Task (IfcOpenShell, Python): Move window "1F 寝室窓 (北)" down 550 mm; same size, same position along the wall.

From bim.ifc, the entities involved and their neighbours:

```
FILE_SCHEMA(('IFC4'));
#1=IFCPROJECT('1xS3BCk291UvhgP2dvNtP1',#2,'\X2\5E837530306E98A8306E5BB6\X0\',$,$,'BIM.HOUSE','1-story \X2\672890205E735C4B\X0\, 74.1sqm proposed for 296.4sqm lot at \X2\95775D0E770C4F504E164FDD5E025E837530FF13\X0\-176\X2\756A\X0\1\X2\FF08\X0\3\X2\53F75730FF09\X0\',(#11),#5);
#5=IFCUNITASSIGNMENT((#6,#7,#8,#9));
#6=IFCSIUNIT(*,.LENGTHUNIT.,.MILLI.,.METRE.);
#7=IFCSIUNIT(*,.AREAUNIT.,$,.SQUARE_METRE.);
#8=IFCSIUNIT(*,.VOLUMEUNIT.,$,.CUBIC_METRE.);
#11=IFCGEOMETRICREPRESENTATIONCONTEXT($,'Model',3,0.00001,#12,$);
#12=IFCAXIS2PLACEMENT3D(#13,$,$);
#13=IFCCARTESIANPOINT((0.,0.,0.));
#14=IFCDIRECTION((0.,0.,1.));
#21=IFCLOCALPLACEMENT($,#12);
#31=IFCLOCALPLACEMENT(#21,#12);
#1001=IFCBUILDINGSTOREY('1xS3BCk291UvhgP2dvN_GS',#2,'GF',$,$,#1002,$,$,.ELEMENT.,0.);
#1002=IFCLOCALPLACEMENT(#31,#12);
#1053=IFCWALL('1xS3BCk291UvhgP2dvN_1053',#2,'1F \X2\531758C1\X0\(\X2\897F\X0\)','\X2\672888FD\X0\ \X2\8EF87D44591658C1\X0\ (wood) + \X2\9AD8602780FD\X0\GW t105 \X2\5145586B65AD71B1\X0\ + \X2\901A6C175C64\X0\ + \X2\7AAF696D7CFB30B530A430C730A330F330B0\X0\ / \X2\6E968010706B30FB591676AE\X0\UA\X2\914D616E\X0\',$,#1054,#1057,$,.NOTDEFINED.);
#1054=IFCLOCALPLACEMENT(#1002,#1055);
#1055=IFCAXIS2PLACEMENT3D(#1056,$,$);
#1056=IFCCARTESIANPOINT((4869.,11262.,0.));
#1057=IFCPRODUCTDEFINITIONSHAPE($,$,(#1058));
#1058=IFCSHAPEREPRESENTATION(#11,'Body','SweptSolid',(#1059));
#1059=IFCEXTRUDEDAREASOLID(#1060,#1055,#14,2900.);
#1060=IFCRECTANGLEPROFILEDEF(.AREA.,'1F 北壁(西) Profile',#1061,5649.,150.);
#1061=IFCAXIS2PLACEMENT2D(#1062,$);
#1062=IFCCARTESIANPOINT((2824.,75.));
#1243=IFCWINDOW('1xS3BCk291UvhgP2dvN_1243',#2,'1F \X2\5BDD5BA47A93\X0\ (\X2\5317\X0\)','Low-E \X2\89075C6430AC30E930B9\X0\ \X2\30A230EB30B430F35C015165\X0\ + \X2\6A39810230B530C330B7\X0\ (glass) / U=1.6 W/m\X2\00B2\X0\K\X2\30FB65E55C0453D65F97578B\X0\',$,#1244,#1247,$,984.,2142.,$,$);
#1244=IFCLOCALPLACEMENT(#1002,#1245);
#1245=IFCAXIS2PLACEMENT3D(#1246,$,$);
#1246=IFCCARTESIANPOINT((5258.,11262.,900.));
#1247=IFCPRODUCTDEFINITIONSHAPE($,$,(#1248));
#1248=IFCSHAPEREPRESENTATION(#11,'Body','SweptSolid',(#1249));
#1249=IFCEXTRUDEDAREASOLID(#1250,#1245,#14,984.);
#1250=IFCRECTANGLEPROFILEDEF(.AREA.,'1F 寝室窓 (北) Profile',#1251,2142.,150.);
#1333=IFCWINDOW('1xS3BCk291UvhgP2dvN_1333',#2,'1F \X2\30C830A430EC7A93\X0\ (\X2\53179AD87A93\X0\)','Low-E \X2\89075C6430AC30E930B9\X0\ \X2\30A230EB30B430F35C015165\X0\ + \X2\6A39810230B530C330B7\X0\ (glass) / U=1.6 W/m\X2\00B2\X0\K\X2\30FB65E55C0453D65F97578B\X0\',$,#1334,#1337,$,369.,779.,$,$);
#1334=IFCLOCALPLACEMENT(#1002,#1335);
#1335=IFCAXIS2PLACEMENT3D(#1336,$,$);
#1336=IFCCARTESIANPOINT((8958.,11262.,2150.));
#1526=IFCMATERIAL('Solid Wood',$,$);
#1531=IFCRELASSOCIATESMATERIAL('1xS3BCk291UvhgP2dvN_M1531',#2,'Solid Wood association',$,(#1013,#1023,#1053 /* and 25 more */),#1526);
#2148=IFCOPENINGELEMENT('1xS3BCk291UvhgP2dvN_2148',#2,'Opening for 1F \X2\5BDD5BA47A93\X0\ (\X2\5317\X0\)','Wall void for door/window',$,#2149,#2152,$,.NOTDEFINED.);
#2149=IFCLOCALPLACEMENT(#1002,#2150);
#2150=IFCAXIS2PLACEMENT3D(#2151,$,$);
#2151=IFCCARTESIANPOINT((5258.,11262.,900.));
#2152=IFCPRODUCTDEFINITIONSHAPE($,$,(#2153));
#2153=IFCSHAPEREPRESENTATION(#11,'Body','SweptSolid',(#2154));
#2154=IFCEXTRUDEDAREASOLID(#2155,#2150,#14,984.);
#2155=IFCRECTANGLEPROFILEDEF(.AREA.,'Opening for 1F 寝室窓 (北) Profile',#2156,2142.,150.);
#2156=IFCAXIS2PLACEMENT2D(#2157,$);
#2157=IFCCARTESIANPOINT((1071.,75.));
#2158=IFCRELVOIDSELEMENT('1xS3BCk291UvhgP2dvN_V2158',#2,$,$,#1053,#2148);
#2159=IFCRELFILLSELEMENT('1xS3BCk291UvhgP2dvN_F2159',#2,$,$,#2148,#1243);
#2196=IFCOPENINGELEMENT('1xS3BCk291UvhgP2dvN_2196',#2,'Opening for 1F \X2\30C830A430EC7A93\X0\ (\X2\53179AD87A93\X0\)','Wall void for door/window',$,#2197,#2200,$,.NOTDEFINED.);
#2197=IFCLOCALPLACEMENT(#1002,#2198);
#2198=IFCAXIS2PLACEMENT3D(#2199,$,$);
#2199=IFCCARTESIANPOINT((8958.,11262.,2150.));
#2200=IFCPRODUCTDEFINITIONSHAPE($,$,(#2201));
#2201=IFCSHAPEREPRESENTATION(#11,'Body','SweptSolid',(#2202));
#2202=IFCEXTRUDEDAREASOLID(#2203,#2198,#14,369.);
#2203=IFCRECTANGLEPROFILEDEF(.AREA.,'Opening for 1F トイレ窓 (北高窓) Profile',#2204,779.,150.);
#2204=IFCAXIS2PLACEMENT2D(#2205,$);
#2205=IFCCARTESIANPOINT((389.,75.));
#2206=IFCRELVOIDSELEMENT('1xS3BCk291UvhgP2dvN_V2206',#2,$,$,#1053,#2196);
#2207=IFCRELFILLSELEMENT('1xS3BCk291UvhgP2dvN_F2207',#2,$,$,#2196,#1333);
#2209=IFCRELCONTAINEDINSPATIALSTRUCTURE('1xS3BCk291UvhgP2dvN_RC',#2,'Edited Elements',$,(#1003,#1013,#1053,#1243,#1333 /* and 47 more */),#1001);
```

```python
import numpy as np
import ifcopenshell
import ifcopenshell.api.geometry
import ifcopenshell.util.placement
import ifcopenshell.util.unit

model = ifcopenshell.open("bim.ifc")
unit_scale = ifcopenshell.util.unit.calculate_unit_scale(model)

window = model.by_guid("1xS3BCk291UvhgP2dvN_1243")
opening = window.FillsVoids[0].RelatingOpeningElement
dz = -0.55 / unit_scale

shift = np.array([0.0, 0.0, dz])
# The window is not placed relative to its opening, so move both.
for product in (opening, window):
    matrix = ifcopenshell.util.placement.get_local_placement(product.ObjectPlacement)
    matrix[:3, 3] += shift
    ifcopenshell.api.geometry.edit_object_placement(model, product=product, matrix=matrix, is_si=False)

print(f"moved by {dz * unit_scale:+.3f} m")

model.write("bim_rev.ifc")
```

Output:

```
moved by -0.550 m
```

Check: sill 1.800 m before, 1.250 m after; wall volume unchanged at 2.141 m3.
